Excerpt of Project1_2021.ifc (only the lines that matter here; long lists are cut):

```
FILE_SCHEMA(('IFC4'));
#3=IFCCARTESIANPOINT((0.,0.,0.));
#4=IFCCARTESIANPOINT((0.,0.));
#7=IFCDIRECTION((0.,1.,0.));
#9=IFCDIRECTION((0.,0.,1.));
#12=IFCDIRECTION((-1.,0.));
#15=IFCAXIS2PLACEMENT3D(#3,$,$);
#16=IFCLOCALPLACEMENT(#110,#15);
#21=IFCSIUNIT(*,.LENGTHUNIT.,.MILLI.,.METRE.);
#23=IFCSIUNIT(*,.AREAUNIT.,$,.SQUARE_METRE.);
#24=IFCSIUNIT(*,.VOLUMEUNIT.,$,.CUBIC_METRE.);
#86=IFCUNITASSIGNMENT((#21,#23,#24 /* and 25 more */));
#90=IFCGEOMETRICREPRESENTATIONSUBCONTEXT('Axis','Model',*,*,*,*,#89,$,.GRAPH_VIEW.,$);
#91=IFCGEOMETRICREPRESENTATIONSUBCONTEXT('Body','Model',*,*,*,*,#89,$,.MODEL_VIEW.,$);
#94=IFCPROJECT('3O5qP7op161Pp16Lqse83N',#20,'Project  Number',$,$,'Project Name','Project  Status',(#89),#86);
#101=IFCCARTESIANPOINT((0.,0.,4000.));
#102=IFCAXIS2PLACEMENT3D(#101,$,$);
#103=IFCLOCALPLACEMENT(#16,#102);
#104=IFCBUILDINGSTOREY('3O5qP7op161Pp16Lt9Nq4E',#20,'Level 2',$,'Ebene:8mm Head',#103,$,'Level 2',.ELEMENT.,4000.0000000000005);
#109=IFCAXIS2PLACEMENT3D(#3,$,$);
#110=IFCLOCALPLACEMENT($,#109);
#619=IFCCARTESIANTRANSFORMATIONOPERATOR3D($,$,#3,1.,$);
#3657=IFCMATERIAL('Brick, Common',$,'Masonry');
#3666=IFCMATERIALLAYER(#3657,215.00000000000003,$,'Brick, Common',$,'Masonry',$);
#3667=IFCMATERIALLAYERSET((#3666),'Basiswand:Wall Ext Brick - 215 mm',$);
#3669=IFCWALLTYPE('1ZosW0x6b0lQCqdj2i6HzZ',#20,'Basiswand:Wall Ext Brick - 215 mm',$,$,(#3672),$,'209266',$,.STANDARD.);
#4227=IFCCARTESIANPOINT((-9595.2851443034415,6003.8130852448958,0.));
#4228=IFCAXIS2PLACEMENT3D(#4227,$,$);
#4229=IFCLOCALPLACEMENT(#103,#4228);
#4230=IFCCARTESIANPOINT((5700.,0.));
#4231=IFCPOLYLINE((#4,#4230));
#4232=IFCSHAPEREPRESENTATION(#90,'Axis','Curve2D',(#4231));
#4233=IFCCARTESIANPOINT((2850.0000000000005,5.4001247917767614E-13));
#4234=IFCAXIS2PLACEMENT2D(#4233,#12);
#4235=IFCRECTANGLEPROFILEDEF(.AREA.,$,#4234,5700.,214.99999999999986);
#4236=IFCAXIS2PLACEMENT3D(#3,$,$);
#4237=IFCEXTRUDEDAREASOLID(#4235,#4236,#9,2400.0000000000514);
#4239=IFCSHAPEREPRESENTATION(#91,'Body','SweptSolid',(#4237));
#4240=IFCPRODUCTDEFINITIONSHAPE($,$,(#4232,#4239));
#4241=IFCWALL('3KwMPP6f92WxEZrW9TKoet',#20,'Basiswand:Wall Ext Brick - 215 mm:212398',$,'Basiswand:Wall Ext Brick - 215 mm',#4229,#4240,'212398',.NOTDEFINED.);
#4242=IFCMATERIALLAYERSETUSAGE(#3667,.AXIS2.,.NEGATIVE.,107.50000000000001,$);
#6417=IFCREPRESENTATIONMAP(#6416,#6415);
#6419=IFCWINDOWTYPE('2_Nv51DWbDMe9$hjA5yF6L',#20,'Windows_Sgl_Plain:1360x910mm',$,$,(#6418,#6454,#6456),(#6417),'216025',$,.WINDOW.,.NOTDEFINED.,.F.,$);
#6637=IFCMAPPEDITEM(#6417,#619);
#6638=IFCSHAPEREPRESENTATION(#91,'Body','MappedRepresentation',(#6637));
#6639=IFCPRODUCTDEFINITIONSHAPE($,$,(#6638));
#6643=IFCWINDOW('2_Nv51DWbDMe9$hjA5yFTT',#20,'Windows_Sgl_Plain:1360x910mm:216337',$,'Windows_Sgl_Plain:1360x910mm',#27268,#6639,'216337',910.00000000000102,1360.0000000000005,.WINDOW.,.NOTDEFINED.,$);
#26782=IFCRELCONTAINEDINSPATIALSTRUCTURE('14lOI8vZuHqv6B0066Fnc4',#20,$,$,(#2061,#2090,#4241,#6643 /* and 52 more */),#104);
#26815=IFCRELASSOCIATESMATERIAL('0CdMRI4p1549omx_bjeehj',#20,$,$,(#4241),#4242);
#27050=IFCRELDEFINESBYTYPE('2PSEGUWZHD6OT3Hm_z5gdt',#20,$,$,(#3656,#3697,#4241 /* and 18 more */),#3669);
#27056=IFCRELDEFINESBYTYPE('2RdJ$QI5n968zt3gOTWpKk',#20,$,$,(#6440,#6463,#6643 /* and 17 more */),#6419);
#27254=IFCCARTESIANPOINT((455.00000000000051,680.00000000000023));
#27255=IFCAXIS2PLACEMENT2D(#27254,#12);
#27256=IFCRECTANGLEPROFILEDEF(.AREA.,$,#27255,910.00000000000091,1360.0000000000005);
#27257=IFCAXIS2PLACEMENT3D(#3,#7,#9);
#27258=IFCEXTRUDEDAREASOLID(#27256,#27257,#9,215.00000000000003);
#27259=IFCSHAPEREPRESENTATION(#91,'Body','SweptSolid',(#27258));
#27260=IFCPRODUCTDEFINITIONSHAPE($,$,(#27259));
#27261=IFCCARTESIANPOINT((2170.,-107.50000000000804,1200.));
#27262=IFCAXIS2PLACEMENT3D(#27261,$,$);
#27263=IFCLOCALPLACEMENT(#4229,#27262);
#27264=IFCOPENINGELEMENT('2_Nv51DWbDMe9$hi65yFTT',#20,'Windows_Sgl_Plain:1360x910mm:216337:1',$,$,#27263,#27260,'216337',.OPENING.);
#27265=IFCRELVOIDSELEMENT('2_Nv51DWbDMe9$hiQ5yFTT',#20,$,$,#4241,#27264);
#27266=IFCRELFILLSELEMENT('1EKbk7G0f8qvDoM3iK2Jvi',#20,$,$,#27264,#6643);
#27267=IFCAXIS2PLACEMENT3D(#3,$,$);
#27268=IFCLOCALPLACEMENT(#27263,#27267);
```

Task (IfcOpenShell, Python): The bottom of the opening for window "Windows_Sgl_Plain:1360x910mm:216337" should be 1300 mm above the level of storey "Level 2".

```python
import numpy as np
import ifcopenshell
import ifcopenshell.api.geometry
import ifcopenshell.geom
import ifcopenshell.util.element
import ifcopenshell.util.placement
import ifcopenshell.util.shape
import ifcopenshell.util.unit

model = ifcopenshell.open("Project1_2021.ifc")
unit_scale = ifcopenshell.util.unit.calculate_unit_scale(model)

window = model.by_guid("2_Nv51DWbDMe9$hjA5yFTT")
opening = window.FillsVoids[0].RelatingOpeningElement
storey = ifcopenshell.util.element.get_container(window, ifc_class="IfcBuildingStorey")
level = ifcopenshell.util.placement.get_local_placement(storey.ObjectPlacement)[2, 3]

# The opening's origin need not be at the sill, so measure its lowest point.
shape = ifcopenshell.geom.create_shape(ifcopenshell.geom.settings(), opening)
bottom = ifcopenshell.util.shape.get_shape_bottom_elevation(shape, shape.geometry) / unit_scale
dz = level + 1.3 / unit_scale - bottom

shift = np.array([0.0, 0.0, dz])
# The window is placed relative to its opening, so it follows when the opening moves.
matrix = ifcopenshell.util.placement.get_local_placement(opening.ObjectPlacement)
matrix[:3, 3] += shift
ifcopenshell.api.geometry.edit_object_placement(
    model, product=opening, matrix=matrix, is_si=False, should_transform_children=True
)

print(f"moved by {dz * unit_scale:+.3f} m")

model.write("Project1_2021-out.ifc")
```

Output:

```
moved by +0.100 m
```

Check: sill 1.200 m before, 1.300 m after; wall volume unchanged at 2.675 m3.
